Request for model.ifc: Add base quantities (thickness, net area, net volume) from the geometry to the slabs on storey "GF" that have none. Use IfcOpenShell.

First a look at what the model holds.

```python
import ifcopenshell
import ifcopenshell.util.element
import ifcopenshell.util.unit

model = ifcopenshell.open("model.ifc")
print(model.schema)
for unit_type in ("LENGTHUNIT", "AREAUNIT", "VOLUMEUNIT"):
    print(unit_type, ifcopenshell.util.unit.calculate_unit_scale(model, unit_type))
storey = next(s for s in model.by_type("IfcBuildingStorey") if s.Name == "GF")
slabs = [e for e in ifcopenshell.util.element.get_decomposition(storey) if e.is_a("IfcSlab")]
for e in sorted(slabs, key=lambda e: e.id()):
    print(e.id(), e.is_a(), e.Name, list(ifcopenshell.util.element.get_psets(e, qtos_only=True)), sep=" | ")
```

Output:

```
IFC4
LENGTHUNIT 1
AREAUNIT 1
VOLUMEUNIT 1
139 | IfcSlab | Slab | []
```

```python
import ifcopenshell
import ifcopenshell.api.pset
import ifcopenshell.geom
import ifcopenshell.util.element
import ifcopenshell.util.shape
import ifcopenshell.util.unit

model = ifcopenshell.open("model.ifc")
unit_scale = ifcopenshell.util.unit.calculate_unit_scale(model)
area_scale = ifcopenshell.util.unit.calculate_unit_scale(model, "AREAUNIT")
volume_scale = ifcopenshell.util.unit.calculate_unit_scale(model, "VOLUMEUNIT")
settings = ifcopenshell.geom.settings()

storey = next(s for s in model.by_type("IfcBuildingStorey") if s.Name == "GF")
slabs = [e for e in ifcopenshell.util.element.get_decomposition(storey) if e.is_a("IfcSlab")]

for e in sorted(slabs, key=lambda e: e.id()):
    if ifcopenshell.util.element.get_psets(e, qtos_only=True, should_inherit=False):
        continue
    # Geometry comes back in metres, in the element's own axes.
    shape = ifcopenshell.geom.create_shape(settings, e)
    values = {
        "Width": ifcopenshell.util.shape.get_z(shape.geometry) / unit_scale,
        "NetArea": ifcopenshell.util.shape.get_footprint_area(shape.geometry) / area_scale,
        "NetVolume": ifcopenshell.util.shape.get_volume(shape.geometry) / volume_scale,
    }
    qto = ifcopenshell.api.pset.add_qto(model, product=e, name="Qto_SlabBaseQuantities")
    ifcopenshell.api.pset.edit_qto(model, qto=qto, properties=values)
    print(e.id(), {k: round(v, 3) for k, v in values.items()})

model.write("model-out.ifc")
```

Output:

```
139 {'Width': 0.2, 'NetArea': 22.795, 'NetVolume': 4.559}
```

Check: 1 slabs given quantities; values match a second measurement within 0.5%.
